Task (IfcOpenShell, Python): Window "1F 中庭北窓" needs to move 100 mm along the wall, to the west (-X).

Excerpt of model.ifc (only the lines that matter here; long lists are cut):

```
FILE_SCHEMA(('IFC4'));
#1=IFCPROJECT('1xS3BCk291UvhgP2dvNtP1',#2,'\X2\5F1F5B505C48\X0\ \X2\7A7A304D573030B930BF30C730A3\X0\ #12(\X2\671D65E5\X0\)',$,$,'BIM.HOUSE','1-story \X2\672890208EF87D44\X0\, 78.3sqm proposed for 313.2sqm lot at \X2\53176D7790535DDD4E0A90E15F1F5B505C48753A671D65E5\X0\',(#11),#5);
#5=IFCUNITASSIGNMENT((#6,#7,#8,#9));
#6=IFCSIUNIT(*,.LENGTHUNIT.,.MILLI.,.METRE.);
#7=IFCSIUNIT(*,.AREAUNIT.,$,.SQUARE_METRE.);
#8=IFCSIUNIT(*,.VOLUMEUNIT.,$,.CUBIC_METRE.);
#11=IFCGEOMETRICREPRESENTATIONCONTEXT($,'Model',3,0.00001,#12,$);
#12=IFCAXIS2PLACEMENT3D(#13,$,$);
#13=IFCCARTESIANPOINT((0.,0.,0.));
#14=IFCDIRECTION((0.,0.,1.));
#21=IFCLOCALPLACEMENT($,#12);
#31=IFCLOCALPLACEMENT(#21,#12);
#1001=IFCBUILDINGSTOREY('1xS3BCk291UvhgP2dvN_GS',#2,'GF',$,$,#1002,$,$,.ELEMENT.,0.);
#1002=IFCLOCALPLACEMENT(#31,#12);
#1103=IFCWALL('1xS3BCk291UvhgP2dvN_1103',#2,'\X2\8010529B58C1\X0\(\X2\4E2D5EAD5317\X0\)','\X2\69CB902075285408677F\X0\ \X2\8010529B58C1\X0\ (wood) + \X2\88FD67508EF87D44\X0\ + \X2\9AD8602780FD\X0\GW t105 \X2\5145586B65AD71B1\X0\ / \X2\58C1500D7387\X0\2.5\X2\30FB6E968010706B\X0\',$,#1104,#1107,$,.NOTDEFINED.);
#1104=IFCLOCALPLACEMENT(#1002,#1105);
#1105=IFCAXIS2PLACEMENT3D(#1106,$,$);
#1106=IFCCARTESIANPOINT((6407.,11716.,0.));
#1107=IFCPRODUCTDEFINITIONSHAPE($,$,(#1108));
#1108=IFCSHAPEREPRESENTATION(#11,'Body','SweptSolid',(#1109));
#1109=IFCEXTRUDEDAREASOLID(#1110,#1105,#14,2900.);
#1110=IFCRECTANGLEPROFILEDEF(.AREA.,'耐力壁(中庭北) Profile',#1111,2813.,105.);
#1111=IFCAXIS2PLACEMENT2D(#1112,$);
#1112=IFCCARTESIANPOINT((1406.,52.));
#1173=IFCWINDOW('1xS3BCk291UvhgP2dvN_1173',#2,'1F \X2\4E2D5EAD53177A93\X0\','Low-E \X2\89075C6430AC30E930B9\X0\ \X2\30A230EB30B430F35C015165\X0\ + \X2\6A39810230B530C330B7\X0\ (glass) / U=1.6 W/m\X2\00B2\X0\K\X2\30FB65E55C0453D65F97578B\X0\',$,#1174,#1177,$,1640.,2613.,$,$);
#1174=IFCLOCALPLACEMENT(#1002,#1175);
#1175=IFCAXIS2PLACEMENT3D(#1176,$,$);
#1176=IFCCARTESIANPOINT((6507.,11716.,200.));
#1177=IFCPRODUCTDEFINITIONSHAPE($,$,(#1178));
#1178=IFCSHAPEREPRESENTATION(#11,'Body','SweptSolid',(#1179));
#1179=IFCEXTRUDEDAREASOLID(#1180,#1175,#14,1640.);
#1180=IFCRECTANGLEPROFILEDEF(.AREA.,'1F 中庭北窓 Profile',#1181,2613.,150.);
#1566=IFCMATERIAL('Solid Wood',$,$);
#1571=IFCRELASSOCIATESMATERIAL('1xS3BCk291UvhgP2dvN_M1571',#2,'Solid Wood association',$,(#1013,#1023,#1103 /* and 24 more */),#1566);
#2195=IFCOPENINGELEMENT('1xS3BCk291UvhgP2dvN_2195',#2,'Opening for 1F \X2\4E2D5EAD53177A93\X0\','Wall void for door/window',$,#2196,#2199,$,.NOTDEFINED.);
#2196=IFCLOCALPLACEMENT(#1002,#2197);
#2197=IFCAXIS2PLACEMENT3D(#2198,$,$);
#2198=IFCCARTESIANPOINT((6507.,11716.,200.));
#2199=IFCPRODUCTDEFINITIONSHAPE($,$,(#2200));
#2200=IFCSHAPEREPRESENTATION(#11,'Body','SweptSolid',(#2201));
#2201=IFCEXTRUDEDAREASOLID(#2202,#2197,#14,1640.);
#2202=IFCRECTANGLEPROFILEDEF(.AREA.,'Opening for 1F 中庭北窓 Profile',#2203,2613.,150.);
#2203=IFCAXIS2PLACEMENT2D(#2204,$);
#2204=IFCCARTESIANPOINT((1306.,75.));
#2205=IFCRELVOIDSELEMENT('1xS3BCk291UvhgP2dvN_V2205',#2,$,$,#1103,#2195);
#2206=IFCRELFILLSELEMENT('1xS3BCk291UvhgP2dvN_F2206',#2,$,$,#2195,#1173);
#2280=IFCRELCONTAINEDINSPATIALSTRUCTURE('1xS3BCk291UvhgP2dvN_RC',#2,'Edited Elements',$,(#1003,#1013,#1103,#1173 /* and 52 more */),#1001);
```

```python
import ifcopenshell
import ifcopenshell.api.geometry
import ifcopenshell.util.placement

model = ifcopenshell.open("model.ifc")

window = model.by_id(1173)
opening = window.FillsVoids[0].RelatingOpeningElement
wall = opening.VoidsElements[0].RelatingBuildingElement

wall_matrix = ifcopenshell.util.placement.get_local_placement(wall.ObjectPlacement)
shift = wall_matrix[:3, 0] * -100.0
before = ifcopenshell.util.placement.get_local_placement(window.ObjectPlacement)[:3, 3].copy()

# The window is not placed relative to its opening, so move both.
for product in (opening, window):
    matrix = ifcopenshell.util.placement.get_local_placement(product.ObjectPlacement)
    matrix[:3, 3] += shift
    ifcopenshell.api.geometry.edit_object_placement(model, product=product, matrix=matrix, is_si=False)

after = ifcopenshell.util.placement.get_local_placement(window.ObjectPlacement)[:3, 3]
print("window moved by", (after - before).round(3) + 0.0)

model.write("model-out.ifc")
```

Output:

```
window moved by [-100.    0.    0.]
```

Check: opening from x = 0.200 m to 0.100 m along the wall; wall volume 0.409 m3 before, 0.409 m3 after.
